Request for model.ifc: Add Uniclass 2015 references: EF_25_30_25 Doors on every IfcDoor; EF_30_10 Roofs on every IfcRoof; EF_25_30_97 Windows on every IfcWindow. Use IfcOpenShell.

First a look at what the model holds.

```python
import ifcopenshell

model = ifcopenshell.open("model.ifc")
print(model.schema)
print("classifications:", [c.Name for c in model.by_type("IfcClassification")])
for ifc_class in ("IfcDoor", "IfcRoof", "IfcStair", "IfcWall", "IfcWindow"):
    print(ifc_class, len(model.by_type(ifc_class)))
```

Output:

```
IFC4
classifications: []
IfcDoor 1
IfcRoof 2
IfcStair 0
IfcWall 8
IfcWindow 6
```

```python
import ifcopenshell
import ifcopenshell.api.classification

model = ifcopenshell.open("model.ifc")

system = ifcopenshell.api.classification.add_classification(model, classification="Uniclass 2015")

codes = {
    "IfcDoor": ("EF_25_30_25", "Doors"),
    "IfcRoof": ("EF_30_10", "Roofs"),
    "IfcWindow": ("EF_25_30_97", "Windows"),
}
for ifc_class, (code, name) in codes.items():
    products = model.by_type(ifc_class)
    ifcopenshell.api.classification.add_reference(
        model, products=products, classification=system, identification=code, name=name
    )
    print(code, len(products))

model.write("model_rev.ifc")
```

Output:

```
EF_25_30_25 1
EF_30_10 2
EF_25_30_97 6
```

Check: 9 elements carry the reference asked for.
